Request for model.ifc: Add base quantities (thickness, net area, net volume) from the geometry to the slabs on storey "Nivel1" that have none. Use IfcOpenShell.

First a look at what the model holds.

```python
import ifcopenshell
import ifcopenshell.util.element
import ifcopenshell.util.unit

model = ifcopenshell.open("model.ifc")
print(model.schema)
for unit_type in ("LENGTHUNIT", "AREAUNIT", "VOLUMEUNIT"):
    print(unit_type, ifcopenshell.util.unit.calculate_unit_scale(model, unit_type))
storey = next(s for s in model.by_type("IfcBuildingStorey") if s.Name == "Nivel1")
slabs = [e for e in ifcopenshell.util.element.get_decomposition(storey) if e.is_a("IfcSlab")]
for e in sorted(slabs, key=lambda e: e.id()):
    print(e.id(), e.is_a(), e.Name, list(ifcopenshell.util.element.get_psets(e, qtos_only=True)), sep=" | ")
```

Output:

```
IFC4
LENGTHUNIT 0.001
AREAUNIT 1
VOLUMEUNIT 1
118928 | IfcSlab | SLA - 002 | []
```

```python
import ifcopenshell
import ifcopenshell.api.pset
import ifcopenshell.geom
import ifcopenshell.util.element
import ifcopenshell.util.shape
import ifcopenshell.util.unit

model = ifcopenshell.open("model.ifc")
unit_scale = ifcopenshell.util.unit.calculate_unit_scale(model)
area_scale = ifcopenshell.util.unit.calculate_unit_scale(model, "AREAUNIT")
volume_scale = ifcopenshell.util.unit.calculate_unit_scale(model, "VOLUMEUNIT")
settings = ifcopenshell.geom.settings()

storey = next(s for s in model.by_type("IfcBuildingStorey") if s.Name == "Nivel1")
slabs = [e for e in ifcopenshell.util.element.get_decomposition(storey) if e.is_a("IfcSlab")]

for e in sorted(slabs, key=lambda e: e.id()):
    if ifcopenshell.util.element.get_psets(e, qtos_only=True, should_inherit=False):
        continue
    # Geometry comes back in metres, in the element's own axes.
    shape = ifcopenshell.geom.create_shape(settings, e)
    values = {
        "Width": ifcopenshell.util.shape.get_z(shape.geometry) / unit_scale,
        "NetArea": ifcopenshell.util.shape.get_footprint_area(shape.geometry) / area_scale,
        "NetVolume": ifcopenshell.util.shape.get_volume(shape.geometry) / volume_scale,
    }
    qto = ifcopenshell.api.pset.add_qto(model, product=e, name="Qto_SlabBaseQuantities")
    ifcopenshell.api.pset.edit_qto(model, qto=qto, properties=values)
    print(e.id(), {k: round(v, 3) for k, v in values.items()})

model.write("model-out.ifc")
```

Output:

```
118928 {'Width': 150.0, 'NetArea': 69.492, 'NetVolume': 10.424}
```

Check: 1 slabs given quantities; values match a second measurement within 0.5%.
